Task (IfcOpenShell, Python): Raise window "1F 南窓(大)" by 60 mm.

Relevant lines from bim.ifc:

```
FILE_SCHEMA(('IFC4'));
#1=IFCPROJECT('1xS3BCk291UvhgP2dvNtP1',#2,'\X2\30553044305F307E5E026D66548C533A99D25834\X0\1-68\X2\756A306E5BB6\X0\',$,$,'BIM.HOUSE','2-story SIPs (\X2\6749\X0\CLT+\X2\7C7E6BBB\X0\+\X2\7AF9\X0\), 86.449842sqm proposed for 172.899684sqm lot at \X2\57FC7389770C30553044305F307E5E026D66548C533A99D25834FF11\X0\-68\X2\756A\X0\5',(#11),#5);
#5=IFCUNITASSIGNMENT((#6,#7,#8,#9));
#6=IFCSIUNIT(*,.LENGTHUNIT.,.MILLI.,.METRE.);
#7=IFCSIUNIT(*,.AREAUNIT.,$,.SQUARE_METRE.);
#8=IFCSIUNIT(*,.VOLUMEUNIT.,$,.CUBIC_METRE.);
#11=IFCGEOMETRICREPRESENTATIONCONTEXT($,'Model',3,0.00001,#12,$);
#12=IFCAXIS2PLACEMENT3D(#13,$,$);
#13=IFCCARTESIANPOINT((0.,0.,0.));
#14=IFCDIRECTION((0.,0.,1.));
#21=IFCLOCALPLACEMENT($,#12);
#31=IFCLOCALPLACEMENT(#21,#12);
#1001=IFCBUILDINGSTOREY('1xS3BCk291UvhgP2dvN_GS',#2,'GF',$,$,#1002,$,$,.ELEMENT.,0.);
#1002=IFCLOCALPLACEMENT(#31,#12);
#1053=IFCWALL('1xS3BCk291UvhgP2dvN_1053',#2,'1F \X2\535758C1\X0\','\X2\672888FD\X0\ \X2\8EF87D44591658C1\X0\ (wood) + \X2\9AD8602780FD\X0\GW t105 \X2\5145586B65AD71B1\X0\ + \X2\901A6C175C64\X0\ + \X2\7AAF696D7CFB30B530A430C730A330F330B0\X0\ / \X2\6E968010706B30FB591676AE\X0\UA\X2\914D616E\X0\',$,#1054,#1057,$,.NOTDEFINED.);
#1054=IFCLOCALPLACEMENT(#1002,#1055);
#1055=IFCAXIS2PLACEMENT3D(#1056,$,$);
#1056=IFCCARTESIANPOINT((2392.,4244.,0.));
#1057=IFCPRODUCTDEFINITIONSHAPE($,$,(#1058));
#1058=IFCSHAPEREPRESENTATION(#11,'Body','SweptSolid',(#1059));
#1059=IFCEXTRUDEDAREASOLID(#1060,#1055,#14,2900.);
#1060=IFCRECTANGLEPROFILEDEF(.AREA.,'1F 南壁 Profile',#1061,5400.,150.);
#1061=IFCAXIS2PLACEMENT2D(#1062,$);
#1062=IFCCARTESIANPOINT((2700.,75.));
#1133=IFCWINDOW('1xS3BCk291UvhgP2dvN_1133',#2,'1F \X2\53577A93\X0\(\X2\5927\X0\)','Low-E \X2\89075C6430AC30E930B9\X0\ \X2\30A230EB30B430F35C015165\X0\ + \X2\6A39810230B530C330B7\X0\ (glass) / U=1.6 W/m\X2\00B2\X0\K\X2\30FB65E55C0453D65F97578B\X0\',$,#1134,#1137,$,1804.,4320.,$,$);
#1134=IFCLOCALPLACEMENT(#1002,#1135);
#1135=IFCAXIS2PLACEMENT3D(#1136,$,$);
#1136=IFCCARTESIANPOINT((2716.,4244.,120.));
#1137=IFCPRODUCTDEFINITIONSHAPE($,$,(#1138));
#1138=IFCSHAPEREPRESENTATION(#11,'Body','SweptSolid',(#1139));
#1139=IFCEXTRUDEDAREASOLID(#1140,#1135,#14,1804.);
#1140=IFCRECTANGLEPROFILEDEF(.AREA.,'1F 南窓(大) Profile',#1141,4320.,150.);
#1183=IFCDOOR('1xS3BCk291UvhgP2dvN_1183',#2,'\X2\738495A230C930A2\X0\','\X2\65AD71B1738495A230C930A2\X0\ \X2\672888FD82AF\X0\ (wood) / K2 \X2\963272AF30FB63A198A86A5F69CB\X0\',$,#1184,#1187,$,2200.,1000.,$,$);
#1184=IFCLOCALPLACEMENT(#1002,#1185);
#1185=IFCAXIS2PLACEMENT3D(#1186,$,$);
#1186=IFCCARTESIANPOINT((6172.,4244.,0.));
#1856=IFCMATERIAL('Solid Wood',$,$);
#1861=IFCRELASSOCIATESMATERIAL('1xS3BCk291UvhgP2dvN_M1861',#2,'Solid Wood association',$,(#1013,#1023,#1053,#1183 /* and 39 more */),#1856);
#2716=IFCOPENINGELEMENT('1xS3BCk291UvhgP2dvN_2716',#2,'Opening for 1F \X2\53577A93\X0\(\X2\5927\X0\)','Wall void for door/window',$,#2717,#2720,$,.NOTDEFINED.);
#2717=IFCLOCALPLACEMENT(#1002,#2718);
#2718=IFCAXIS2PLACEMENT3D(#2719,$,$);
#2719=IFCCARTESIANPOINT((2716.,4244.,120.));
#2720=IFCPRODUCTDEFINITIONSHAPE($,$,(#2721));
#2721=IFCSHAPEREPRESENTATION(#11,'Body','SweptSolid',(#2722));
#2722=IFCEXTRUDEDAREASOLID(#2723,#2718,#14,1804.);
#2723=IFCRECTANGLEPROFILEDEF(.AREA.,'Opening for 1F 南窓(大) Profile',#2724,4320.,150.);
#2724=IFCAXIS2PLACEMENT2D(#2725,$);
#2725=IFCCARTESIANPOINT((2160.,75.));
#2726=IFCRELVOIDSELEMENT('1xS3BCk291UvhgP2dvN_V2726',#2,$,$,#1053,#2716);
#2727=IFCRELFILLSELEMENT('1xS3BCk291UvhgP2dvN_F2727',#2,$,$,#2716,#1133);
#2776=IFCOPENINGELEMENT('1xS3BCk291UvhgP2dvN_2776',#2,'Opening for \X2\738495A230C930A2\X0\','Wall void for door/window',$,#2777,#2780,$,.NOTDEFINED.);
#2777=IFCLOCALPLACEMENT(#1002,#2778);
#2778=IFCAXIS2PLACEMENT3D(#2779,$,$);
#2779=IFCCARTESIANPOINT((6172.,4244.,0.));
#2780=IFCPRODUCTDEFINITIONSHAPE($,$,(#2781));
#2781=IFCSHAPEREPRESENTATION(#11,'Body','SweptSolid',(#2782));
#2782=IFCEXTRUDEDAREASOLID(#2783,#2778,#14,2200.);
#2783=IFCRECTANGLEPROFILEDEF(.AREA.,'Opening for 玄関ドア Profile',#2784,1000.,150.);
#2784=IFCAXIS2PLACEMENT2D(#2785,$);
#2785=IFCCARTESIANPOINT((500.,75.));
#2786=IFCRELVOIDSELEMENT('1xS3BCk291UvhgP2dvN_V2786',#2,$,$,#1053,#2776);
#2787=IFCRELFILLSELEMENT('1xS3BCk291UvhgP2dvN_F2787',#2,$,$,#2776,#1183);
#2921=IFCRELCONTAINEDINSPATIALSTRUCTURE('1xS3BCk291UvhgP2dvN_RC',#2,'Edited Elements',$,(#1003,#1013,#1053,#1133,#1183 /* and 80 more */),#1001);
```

```python
import numpy as np
import ifcopenshell
import ifcopenshell.api.geometry
import ifcopenshell.util.placement
import ifcopenshell.util.unit

model = ifcopenshell.open("bim.ifc")
unit_scale = ifcopenshell.util.unit.calculate_unit_scale(model)

window = model.by_guid("1xS3BCk291UvhgP2dvN_1133")
opening = window.FillsVoids[0].RelatingOpeningElement
dz = 0.06 / unit_scale

shift = np.array([0.0, 0.0, dz])
# The window is not placed relative to its opening, so move both.
for product in (opening, window):
    matrix = ifcopenshell.util.placement.get_local_placement(product.ObjectPlacement)
    matrix[:3, 3] += shift
    ifcopenshell.api.geometry.edit_object_placement(model, product=product, matrix=matrix, is_si=False)

print(f"moved by {dz * unit_scale:+.3f} m")

model.write("bim_updated.ifc")
```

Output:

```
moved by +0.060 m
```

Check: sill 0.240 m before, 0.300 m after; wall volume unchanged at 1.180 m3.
